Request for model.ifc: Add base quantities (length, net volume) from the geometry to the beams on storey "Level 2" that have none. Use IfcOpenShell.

First a look at what the model holds.

```python
import ifcopenshell
import ifcopenshell.util.element
import ifcopenshell.util.unit

model = ifcopenshell.open("model.ifc")
print(model.schema)
for unit_type in ("LENGTHUNIT", "AREAUNIT", "VOLUMEUNIT"):
    print(unit_type, ifcopenshell.util.unit.calculate_unit_scale(model, unit_type))
storey = next(s for s in model.by_type("IfcBuildingStorey") if s.Name == "Level 2")
beams = [e for e in ifcopenshell.util.element.get_decomposition(storey) if e.is_a("IfcBeam")]
for e in sorted(beams, key=lambda e: e.id()):
    print(e.id(), e.is_a(), e.Name, list(ifcopenshell.util.element.get_psets(e, qtos_only=True)), sep=" | ")
```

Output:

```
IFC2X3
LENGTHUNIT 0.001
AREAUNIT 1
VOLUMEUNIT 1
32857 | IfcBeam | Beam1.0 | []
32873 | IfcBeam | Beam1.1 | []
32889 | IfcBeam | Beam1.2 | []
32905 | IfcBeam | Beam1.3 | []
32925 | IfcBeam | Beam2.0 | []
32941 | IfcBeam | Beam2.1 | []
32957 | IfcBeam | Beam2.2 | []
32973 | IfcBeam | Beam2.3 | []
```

```python
import ifcopenshell
import ifcopenshell.api.pset
import ifcopenshell.geom
import ifcopenshell.util.element
import ifcopenshell.util.shape
import ifcopenshell.util.unit

model = ifcopenshell.open("model.ifc")
unit_scale = ifcopenshell.util.unit.calculate_unit_scale(model)
volume_scale = ifcopenshell.util.unit.calculate_unit_scale(model, "VOLUMEUNIT")
settings = ifcopenshell.geom.settings()

storey = next(s for s in model.by_type("IfcBuildingStorey") if s.Name == "Level 2")
beams = [e for e in ifcopenshell.util.element.get_decomposition(storey) if e.is_a("IfcBeam")]

for e in sorted(beams, key=lambda e: e.id()):
    if ifcopenshell.util.element.get_psets(e, qtos_only=True, should_inherit=False):
        continue
    # Geometry comes back in metres, in the element's own axes.
    shape = ifcopenshell.geom.create_shape(settings, e)
    values = {
        "Length": ifcopenshell.util.shape.get_max_xyz(shape.geometry) / unit_scale,
        "NetVolume": ifcopenshell.util.shape.get_volume(shape.geometry) / volume_scale,
    }
    qto = ifcopenshell.api.pset.add_qto(model, product=e, name="BaseQuantities")
    ifcopenshell.api.pset.edit_qto(model, qto=qto, properties=values)
    print(e.id(), {k: round(v, 3) for k, v in values.items()})

model.write("model_v2.ifc")
```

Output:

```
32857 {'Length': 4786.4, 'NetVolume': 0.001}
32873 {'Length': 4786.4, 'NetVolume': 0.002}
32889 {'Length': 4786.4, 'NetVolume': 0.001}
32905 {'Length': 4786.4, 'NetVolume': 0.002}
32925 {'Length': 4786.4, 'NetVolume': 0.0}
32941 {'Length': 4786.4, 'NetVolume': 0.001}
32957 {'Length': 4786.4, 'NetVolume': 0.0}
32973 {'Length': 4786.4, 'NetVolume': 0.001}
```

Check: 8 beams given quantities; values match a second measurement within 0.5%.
